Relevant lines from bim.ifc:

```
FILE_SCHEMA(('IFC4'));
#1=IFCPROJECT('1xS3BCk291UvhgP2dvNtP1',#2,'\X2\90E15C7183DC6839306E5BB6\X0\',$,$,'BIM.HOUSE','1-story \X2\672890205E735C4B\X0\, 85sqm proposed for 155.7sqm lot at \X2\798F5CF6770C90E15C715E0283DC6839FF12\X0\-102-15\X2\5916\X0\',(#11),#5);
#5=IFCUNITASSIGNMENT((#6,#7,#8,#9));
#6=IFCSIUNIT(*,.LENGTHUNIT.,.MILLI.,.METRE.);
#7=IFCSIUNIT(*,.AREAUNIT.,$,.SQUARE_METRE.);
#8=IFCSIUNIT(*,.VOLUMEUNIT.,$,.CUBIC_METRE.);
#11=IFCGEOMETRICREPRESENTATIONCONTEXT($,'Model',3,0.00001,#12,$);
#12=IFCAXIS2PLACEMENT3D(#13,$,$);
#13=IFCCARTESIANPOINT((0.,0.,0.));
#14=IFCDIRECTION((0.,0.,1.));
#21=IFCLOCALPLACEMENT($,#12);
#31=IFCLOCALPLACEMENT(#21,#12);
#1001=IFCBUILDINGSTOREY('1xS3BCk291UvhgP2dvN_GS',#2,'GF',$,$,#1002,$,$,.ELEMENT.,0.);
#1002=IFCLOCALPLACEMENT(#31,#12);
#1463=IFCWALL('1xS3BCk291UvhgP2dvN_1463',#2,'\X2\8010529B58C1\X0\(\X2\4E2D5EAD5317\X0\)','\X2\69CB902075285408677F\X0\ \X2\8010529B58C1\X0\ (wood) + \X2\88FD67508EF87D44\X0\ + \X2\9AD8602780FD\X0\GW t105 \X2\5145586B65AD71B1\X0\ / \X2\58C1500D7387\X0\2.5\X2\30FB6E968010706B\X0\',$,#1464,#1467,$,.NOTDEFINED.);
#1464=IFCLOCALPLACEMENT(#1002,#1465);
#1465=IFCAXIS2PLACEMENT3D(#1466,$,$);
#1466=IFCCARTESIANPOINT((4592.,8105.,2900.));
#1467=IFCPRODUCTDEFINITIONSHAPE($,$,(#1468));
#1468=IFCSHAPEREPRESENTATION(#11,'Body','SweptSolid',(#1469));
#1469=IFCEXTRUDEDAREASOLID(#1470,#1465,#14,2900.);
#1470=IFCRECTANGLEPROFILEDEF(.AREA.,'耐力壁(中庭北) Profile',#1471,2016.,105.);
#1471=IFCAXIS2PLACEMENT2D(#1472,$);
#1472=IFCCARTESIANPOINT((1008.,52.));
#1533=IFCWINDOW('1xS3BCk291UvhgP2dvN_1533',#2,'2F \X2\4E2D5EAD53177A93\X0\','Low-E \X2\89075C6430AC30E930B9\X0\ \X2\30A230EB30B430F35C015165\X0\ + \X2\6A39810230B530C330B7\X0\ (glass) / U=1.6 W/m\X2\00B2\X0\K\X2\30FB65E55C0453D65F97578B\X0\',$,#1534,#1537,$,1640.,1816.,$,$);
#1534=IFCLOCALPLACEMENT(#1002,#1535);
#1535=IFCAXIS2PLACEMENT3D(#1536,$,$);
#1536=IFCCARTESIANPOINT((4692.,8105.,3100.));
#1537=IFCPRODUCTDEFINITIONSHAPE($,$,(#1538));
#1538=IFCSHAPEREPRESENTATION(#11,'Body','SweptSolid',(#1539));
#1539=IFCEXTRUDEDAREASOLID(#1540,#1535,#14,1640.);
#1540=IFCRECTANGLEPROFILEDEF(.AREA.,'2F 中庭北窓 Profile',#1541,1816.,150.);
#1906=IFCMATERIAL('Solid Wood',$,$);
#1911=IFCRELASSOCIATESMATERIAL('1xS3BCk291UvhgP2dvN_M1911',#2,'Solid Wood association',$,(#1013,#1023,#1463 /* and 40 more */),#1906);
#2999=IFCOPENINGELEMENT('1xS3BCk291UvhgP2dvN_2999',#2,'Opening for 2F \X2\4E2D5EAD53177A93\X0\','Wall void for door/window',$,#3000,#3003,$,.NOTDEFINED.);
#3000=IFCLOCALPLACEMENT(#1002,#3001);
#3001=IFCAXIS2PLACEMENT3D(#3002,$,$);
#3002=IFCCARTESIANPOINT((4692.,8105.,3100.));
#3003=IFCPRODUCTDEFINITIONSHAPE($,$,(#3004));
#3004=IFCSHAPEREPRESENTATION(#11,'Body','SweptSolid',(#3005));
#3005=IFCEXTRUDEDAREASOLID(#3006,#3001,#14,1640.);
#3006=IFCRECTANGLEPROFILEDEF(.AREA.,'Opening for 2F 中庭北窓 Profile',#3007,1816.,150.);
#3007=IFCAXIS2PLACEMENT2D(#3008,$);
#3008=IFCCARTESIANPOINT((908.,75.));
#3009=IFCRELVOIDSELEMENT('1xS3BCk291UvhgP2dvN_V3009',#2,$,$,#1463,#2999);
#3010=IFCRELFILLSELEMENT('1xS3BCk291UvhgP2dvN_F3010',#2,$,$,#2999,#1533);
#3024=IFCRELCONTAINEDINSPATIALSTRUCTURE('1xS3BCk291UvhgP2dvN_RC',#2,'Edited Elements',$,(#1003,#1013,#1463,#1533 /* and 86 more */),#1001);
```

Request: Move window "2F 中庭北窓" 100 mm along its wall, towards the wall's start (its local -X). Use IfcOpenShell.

```python
import ifcopenshell
import ifcopenshell.api.geometry
import ifcopenshell.util.placement
import ifcopenshell.util.unit

model = ifcopenshell.open("bim.ifc")
unit_scale = ifcopenshell.util.unit.calculate_unit_scale(model)

window = model.by_guid("1xS3BCk291UvhgP2dvN_1533")
opening = window.FillsVoids[0].RelatingOpeningElement
wall = opening.VoidsElements[0].RelatingBuildingElement

wall_matrix = ifcopenshell.util.placement.get_local_placement(wall.ObjectPlacement)
shift = wall_matrix[:3, 0] * -0.1 / unit_scale
before = ifcopenshell.util.placement.get_local_placement(window.ObjectPlacement)[:3, 3].copy()

# The window is not placed relative to its opening, so move both.
for product in (opening, window):
    matrix = ifcopenshell.util.placement.get_local_placement(product.ObjectPlacement)
    matrix[:3, 3] += shift
    ifcopenshell.api.geometry.edit_object_placement(model, product=product, matrix=matrix, is_si=False)

after = ifcopenshell.util.placement.get_local_placement(window.ObjectPlacement)[:3, 3]
print("window moved by", (after - before).round(3) + 0.0)

model.write("bim_rev.ifc")
```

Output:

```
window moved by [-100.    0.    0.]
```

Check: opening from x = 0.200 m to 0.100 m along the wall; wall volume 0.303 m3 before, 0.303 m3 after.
